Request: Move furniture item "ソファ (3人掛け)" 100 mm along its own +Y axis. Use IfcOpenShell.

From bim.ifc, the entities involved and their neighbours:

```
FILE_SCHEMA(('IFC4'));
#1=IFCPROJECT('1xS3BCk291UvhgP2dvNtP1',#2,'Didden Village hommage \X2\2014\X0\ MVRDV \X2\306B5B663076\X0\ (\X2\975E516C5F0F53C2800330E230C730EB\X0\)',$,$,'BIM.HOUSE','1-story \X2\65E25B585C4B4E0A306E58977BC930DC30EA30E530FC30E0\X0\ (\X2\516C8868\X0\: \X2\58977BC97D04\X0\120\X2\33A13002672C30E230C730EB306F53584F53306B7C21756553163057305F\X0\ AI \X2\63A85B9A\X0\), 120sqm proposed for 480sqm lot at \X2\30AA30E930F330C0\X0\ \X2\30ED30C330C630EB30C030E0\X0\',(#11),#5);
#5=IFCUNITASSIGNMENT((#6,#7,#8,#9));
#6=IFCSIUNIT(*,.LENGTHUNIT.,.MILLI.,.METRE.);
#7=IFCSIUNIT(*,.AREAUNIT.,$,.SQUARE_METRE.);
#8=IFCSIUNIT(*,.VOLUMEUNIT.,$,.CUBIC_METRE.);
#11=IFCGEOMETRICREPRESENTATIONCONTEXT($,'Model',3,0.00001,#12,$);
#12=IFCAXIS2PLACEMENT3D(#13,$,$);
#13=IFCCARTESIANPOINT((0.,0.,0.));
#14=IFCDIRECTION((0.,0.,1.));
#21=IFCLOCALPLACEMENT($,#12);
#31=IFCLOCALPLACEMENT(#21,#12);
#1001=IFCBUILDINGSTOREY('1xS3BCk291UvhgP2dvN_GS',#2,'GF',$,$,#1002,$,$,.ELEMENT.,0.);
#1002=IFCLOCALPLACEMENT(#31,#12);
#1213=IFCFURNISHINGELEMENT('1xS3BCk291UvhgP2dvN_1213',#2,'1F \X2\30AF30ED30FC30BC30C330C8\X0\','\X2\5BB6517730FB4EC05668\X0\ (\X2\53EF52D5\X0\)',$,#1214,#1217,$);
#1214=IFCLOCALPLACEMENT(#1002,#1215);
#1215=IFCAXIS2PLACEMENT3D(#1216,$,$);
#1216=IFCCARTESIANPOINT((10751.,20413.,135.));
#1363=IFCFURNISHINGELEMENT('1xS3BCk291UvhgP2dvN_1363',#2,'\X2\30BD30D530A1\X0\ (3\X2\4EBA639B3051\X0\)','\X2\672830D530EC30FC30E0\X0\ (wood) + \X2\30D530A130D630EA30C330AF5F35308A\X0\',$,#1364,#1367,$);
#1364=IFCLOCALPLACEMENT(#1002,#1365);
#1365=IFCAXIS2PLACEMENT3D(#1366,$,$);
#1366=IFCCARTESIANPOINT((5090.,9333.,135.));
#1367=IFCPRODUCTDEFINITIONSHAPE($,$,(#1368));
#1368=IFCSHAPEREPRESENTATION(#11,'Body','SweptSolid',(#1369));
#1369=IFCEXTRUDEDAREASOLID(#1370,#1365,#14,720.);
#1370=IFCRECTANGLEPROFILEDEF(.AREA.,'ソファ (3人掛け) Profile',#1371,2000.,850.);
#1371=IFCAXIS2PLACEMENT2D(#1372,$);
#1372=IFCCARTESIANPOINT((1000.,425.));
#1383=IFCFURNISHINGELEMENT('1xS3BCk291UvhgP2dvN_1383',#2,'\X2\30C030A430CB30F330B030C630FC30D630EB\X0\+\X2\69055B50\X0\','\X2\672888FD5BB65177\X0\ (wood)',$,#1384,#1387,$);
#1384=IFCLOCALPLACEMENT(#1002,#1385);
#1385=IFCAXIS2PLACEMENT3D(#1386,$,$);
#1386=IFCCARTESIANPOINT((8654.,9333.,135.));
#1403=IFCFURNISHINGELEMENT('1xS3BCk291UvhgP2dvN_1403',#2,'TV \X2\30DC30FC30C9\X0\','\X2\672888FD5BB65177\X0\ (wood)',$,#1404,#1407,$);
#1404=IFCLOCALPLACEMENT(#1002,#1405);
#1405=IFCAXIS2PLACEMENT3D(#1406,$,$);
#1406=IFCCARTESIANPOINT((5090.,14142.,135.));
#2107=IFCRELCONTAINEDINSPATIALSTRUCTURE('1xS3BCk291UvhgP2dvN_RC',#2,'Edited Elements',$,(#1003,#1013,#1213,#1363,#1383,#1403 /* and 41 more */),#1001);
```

```python
import ifcopenshell
import ifcopenshell.api.geometry
import ifcopenshell.util.placement

model = ifcopenshell.open("bim.ifc")

item = model.by_guid("1xS3BCk291UvhgP2dvN_1363")
matrix = ifcopenshell.util.placement.get_local_placement(item.ObjectPlacement)
matrix[:3, 3] += matrix[:3, 1] * 100.0
ifcopenshell.api.geometry.edit_object_placement(model, product=item, matrix=matrix, is_si=False)

print(ifcopenshell.util.placement.get_local_placement(item.ObjectPlacement).round(3) + 0.0)

model.write("bim_v2.ifc")
```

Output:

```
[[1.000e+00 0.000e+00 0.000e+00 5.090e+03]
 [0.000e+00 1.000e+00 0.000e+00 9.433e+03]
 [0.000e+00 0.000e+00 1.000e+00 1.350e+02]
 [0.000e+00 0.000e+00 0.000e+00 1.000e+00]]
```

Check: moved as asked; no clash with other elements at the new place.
